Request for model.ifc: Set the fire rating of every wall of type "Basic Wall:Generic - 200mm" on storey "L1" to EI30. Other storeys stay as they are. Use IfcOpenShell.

First a look at what the model holds.

```python
import ifcopenshell
import ifcopenshell.util.element

model = ifcopenshell.open("model.ifc")
print(model.schema)
storey = next(s for s in model.by_type("IfcBuildingStorey") if s.Name == "L1")
walls = [e for e in ifcopenshell.util.element.get_decomposition(storey) if e.is_a("IfcWall")]
seen = {}
for e in walls:
    element_type = ifcopenshell.util.element.get_type(e)
    key = (element_type.Name if element_type != e and element_type else None, ifcopenshell.util.element.get_pset(e, "Pset_WallCommon", "FireRating"))
    seen[key] = seen.get(key, 0) + 1
for (name, value), count in sorted(seen.items(), key=str):
    print(count, "x", name, "|", value)
```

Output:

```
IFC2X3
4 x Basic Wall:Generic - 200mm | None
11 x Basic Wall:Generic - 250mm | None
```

```python
import ifcopenshell
import ifcopenshell.api.pset
import ifcopenshell.util.element

model = ifcopenshell.open("model.ifc")

storey = next(s for s in model.by_type("IfcBuildingStorey") if s.Name == "L1")
walls = [e for e in ifcopenshell.util.element.get_decomposition(storey) if e.is_a("IfcWall")]

count = 0
for e in walls:
    element_type = ifcopenshell.util.element.get_type(e)
    if element_type in (None, e) or element_type.Name != "Basic Wall:Generic - 200mm":
        continue
    # add_pset returns the element's existing set when there is one.
    pset = ifcopenshell.api.pset.add_pset(model, product=e, name="Pset_WallCommon")
    ifcopenshell.api.pset.edit_pset(model, pset=pset, properties={"FireRating": "EI30"})
    count += 1

print(count, "walls updated")

model.write("model_edited.ifc")
```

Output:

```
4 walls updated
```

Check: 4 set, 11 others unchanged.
